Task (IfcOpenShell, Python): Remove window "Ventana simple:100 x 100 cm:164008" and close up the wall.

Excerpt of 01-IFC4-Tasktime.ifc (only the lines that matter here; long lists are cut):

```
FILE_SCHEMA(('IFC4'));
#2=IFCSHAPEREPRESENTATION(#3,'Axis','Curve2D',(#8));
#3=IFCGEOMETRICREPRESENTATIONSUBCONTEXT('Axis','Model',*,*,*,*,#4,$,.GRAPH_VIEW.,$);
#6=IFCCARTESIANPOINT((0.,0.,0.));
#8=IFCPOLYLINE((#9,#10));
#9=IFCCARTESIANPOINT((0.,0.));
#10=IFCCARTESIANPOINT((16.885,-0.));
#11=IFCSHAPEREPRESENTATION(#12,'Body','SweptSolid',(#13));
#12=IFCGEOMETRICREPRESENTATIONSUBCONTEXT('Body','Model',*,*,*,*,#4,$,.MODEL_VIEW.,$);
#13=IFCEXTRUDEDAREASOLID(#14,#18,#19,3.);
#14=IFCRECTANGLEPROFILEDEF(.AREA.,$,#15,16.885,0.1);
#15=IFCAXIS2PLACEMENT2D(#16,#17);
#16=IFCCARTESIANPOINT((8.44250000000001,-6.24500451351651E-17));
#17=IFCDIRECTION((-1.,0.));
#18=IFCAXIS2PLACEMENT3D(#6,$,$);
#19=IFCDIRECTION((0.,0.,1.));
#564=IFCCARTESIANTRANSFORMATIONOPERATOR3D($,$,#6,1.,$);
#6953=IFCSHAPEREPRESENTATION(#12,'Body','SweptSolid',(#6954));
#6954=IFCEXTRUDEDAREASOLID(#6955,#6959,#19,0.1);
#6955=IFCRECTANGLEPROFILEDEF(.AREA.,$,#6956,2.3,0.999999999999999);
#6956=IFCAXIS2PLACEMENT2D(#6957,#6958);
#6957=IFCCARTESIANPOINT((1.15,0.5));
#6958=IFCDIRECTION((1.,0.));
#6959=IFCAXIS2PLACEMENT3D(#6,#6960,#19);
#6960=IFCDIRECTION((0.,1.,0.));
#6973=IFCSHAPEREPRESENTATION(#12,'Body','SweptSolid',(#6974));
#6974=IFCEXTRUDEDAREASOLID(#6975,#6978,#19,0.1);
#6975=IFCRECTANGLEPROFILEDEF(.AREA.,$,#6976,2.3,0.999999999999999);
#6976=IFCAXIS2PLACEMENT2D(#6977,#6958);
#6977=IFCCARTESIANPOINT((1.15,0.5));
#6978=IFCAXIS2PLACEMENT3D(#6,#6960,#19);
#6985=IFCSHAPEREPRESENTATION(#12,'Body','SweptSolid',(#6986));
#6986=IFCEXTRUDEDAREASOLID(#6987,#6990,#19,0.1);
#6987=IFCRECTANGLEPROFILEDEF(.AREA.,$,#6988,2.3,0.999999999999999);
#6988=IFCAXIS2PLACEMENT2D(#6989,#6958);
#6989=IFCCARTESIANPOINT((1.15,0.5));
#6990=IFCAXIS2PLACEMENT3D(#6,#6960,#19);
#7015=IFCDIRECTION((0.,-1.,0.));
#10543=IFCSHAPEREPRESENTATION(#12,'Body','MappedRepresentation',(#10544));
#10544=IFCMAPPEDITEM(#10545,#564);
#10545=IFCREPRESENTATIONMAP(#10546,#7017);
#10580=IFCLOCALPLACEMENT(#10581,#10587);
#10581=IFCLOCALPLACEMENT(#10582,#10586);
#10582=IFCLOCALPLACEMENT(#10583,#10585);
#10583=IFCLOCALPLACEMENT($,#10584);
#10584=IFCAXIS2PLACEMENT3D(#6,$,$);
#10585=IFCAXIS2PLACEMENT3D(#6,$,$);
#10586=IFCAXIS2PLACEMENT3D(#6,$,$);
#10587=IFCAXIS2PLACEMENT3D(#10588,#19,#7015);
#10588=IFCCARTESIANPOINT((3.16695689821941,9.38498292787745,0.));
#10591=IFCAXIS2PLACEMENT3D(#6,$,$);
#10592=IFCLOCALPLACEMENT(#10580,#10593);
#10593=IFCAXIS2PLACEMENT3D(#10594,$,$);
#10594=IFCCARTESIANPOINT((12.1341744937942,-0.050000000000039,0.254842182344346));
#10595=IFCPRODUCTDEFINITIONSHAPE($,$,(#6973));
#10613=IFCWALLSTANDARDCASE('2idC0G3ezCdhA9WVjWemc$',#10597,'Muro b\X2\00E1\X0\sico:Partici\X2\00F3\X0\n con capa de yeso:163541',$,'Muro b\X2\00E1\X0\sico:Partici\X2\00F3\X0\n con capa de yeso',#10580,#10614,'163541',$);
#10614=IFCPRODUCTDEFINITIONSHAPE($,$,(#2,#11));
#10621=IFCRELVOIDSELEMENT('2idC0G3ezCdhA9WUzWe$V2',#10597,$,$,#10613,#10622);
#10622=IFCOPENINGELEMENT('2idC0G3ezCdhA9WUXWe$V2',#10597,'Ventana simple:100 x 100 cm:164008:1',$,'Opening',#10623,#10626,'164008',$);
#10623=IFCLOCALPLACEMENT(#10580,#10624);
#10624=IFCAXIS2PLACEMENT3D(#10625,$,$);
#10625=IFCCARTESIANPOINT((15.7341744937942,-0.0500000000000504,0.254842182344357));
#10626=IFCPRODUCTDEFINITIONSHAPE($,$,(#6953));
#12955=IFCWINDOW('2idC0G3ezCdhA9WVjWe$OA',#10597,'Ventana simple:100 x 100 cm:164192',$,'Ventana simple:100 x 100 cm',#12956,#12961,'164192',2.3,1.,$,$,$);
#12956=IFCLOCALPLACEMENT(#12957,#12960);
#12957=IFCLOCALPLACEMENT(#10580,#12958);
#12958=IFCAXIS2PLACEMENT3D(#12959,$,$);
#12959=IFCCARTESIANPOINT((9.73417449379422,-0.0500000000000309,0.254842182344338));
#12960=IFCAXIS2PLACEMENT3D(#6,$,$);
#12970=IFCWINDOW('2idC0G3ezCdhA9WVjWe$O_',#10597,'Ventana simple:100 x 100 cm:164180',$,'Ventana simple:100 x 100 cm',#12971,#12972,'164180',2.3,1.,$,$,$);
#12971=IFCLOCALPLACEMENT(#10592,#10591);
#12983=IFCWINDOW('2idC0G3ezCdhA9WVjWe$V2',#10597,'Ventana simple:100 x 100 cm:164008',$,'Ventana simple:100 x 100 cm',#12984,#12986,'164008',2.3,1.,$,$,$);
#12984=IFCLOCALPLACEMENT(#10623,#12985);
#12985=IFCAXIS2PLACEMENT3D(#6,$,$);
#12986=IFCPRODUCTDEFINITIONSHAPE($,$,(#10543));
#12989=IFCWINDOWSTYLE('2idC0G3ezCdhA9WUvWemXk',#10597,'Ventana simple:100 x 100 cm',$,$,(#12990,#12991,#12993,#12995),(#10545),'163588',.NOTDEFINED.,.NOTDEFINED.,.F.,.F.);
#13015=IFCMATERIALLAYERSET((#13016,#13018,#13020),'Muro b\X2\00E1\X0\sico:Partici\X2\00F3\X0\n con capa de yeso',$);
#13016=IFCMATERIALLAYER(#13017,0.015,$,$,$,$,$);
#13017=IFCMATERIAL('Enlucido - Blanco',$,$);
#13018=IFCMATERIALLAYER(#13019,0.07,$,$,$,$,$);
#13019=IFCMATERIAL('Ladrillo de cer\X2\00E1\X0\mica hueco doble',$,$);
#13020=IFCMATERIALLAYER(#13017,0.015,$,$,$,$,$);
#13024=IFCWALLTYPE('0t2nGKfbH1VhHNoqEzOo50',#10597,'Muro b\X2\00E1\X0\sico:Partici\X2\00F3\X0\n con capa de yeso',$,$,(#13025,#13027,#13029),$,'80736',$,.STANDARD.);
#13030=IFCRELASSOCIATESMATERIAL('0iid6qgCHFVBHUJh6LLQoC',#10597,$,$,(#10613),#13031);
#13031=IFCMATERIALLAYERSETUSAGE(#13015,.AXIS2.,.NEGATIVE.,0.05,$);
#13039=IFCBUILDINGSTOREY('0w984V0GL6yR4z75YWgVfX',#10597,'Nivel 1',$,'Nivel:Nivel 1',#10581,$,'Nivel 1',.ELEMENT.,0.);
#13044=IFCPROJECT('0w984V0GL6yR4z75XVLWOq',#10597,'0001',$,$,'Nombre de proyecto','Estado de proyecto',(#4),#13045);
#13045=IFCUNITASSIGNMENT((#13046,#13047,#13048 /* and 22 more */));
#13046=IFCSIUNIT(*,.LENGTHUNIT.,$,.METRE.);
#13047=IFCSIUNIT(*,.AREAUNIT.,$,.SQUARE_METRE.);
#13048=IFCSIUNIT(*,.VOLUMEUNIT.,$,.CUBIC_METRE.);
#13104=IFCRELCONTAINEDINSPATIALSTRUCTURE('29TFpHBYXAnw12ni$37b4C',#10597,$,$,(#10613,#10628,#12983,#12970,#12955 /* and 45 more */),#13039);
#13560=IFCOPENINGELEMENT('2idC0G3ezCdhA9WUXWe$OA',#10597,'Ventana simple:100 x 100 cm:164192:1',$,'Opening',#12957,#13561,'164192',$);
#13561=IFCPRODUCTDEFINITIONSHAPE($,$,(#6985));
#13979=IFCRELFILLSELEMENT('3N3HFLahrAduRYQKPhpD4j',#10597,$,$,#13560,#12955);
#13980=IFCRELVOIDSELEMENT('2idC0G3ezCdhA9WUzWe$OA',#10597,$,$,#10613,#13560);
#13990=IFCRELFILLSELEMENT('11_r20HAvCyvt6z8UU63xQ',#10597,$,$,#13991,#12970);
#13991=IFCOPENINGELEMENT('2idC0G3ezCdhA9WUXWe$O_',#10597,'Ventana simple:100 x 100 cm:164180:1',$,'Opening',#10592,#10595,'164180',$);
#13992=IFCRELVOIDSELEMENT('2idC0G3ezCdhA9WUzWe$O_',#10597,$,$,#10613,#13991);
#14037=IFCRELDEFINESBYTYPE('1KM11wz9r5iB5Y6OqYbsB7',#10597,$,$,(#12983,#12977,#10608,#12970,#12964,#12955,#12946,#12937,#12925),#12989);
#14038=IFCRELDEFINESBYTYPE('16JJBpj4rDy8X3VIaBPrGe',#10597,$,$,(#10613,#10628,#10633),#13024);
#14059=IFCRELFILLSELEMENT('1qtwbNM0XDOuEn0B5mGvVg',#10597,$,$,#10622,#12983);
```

```python
import ifcopenshell
import ifcopenshell.api.feature
import ifcopenshell.api.root
import ifcopenshell.geom
import ifcopenshell.util.shape

model = ifcopenshell.open("01-IFC4-Tasktime.ifc")
settings = ifcopenshell.geom.settings()


def volume(element):
    """Net volume in cubic metres, openings subtracted."""
    shape = ifcopenshell.geom.create_shape(settings, element)
    return ifcopenshell.util.shape.get_volume(shape.geometry)


window = model.by_id(12983)
opening = window.FillsVoids[0].RelatingOpeningElement
wall = opening.VoidsElements[0].RelatingBuildingElement
before = volume(wall)

ifcopenshell.api.root.remove_product(model, product=window)
ifcopenshell.api.feature.remove_feature(model, feature=opening)

after = volume(wall)

print(f"wall volume {before:.3f} -> {after:.3f} m3")

model.write("01-IFC4-Tasktime-out.ifc")
```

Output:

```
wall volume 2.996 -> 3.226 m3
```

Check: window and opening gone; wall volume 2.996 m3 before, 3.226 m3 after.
